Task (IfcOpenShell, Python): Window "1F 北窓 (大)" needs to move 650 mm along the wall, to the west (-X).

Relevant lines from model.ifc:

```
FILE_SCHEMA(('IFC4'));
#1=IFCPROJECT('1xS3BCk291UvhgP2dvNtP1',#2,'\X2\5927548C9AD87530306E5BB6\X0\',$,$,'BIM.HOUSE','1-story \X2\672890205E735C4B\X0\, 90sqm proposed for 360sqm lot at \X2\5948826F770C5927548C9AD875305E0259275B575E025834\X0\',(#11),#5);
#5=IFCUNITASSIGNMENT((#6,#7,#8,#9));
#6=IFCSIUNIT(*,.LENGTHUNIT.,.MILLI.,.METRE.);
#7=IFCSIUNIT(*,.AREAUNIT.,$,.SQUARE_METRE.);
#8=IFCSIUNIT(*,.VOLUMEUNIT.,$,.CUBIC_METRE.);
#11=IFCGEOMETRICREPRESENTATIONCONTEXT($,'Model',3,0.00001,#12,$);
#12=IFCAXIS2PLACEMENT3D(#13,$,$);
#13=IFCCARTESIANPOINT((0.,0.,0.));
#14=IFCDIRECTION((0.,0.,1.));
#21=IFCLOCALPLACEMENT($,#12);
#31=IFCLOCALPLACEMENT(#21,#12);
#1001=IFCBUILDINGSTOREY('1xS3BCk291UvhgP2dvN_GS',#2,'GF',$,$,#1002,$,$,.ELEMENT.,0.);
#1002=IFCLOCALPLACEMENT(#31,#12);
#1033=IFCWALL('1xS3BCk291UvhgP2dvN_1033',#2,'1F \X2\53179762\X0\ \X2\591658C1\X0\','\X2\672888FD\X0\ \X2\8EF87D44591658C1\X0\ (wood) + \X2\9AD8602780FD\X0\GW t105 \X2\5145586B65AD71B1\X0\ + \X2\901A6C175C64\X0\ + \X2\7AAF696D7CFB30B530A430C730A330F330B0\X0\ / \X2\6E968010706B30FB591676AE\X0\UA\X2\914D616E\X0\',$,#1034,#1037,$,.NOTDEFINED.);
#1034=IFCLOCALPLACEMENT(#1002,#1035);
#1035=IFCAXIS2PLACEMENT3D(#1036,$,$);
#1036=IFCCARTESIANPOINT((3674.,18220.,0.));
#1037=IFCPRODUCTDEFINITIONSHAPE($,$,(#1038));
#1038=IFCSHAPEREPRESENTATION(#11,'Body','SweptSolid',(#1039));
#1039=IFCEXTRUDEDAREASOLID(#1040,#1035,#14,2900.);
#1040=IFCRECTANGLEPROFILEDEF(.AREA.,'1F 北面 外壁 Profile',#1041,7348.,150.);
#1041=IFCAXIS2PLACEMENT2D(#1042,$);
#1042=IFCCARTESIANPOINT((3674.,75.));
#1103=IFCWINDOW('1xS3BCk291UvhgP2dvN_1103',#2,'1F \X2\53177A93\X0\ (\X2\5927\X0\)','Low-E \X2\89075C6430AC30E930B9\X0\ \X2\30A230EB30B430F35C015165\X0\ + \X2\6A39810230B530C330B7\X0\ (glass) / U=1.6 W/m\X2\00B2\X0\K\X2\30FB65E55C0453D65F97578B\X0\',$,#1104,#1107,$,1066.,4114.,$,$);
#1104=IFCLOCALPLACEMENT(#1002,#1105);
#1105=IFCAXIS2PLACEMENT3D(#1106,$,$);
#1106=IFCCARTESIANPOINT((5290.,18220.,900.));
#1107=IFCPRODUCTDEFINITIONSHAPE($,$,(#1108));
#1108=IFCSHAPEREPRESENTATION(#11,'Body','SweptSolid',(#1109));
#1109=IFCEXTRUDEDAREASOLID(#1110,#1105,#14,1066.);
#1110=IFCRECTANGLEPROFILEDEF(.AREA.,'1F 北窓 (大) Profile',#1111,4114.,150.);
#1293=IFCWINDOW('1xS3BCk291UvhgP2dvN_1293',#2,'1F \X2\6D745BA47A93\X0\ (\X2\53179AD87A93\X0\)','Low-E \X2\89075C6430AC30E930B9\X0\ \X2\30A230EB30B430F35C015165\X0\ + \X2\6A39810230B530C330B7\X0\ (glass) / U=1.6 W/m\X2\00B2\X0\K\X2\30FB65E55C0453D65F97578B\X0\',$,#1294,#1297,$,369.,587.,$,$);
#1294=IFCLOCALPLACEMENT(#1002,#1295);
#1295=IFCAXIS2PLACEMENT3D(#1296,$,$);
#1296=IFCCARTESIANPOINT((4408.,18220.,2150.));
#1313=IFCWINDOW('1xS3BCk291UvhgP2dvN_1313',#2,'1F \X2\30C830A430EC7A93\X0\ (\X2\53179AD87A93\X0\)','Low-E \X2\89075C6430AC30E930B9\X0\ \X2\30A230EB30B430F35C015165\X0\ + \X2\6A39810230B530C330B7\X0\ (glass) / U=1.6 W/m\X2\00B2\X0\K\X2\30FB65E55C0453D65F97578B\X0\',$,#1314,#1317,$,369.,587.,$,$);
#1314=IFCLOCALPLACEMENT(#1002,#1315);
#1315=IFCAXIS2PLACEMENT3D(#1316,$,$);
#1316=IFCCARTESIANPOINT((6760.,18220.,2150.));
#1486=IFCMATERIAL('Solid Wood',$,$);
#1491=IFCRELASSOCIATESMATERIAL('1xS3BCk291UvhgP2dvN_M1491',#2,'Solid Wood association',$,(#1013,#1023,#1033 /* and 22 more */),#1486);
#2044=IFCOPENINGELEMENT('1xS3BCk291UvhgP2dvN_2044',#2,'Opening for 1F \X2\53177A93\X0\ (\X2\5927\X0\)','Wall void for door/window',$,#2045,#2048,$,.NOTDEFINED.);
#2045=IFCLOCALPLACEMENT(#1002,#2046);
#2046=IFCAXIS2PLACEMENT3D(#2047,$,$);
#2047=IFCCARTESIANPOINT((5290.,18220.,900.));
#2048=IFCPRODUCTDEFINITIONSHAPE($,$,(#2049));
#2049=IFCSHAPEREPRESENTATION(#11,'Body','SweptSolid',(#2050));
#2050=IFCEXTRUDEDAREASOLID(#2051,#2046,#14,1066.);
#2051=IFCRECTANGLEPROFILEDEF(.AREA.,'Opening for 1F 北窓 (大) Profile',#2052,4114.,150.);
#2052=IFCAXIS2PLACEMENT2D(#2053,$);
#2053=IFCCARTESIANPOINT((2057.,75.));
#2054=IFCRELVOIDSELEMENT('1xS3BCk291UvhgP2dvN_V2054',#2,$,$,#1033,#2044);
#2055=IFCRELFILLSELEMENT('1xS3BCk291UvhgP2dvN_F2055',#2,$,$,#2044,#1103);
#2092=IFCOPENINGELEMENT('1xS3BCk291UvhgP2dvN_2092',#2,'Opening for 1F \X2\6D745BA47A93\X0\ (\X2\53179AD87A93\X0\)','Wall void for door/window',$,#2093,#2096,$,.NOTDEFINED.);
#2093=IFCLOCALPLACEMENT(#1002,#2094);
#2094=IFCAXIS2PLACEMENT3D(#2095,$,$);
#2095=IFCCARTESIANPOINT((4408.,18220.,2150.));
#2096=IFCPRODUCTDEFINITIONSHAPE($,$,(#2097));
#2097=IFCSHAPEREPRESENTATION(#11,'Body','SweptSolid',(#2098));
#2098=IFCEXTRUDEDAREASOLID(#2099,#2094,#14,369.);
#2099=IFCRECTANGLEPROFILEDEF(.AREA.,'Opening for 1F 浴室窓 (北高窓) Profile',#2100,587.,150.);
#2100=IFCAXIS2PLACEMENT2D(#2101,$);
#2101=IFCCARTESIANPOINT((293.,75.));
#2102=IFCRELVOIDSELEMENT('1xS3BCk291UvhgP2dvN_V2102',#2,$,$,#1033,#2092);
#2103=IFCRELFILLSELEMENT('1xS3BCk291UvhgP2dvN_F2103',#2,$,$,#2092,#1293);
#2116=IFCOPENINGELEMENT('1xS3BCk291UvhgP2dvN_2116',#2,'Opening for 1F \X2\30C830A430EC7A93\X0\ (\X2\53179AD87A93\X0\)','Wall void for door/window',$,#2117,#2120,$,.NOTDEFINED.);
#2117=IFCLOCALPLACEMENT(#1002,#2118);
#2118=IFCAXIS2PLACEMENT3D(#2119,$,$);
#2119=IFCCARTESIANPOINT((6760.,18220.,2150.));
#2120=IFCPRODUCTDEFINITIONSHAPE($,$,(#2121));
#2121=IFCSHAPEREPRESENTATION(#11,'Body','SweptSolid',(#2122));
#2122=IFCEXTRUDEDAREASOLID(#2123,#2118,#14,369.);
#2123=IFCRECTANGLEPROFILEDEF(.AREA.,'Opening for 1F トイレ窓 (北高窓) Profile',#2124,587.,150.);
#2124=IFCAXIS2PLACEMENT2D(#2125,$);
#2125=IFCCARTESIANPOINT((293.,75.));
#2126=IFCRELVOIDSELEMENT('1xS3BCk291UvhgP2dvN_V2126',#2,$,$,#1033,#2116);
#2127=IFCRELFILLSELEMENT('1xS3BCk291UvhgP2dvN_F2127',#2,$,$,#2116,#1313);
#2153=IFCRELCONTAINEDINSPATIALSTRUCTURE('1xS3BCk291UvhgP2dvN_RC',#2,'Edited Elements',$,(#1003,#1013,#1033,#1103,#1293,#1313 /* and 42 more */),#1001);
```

```python
import ifcopenshell
import ifcopenshell.api.geometry
import ifcopenshell.util.placement

model = ifcopenshell.open("model.ifc")

window = model.by_guid("1xS3BCk291UvhgP2dvN_1103")
opening = window.FillsVoids[0].RelatingOpeningElement
wall = opening.VoidsElements[0].RelatingBuildingElement

wall_matrix = ifcopenshell.util.placement.get_local_placement(wall.ObjectPlacement)
shift = wall_matrix[:3, 0] * -650.0
before = ifcopenshell.util.placement.get_local_placement(window.ObjectPlacement)[:3, 3].copy()

# The window is not placed relative to its opening, so move both.
for product in (opening, window):
    matrix = ifcopenshell.util.placement.get_local_placement(product.ObjectPlacement)
    matrix[:3, 3] += shift
    ifcopenshell.api.geometry.edit_object_placement(model, product=product, matrix=matrix, is_si=False)

after = ifcopenshell.util.placement.get_local_placement(window.ObjectPlacement)[:3, 3]
print("window moved by", (after - before).round(3) + 0.0)

model.write("model_rev.ifc")
```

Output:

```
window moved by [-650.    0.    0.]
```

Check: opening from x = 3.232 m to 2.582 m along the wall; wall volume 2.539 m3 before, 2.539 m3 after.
